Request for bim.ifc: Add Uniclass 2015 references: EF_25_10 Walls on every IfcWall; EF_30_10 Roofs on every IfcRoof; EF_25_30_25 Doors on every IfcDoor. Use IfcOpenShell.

First a look at what the model holds.

```python
import ifcopenshell

model = ifcopenshell.open("bim.ifc")
print(model.schema)
print("classifications:", [c.Name for c in model.by_type("IfcClassification")])
for ifc_class in ("IfcDoor", "IfcRoof", "IfcStair", "IfcWall", "IfcWindow"):
    print(ifc_class, len(model.by_type(ifc_class)))
```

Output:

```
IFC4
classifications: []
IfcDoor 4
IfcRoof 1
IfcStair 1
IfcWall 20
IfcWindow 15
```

```python
import ifcopenshell
import ifcopenshell.api.classification

model = ifcopenshell.open("bim.ifc")

system = ifcopenshell.api.classification.add_classification(model, classification="Uniclass 2015")

codes = {
    "IfcWall": ("EF_25_10", "Walls"),
    "IfcRoof": ("EF_30_10", "Roofs"),
    "IfcDoor": ("EF_25_30_25", "Doors"),
}
for ifc_class, (code, name) in codes.items():
    products = model.by_type(ifc_class)
    ifcopenshell.api.classification.add_reference(
        model, products=products, classification=system, identification=code, name=name
    )
    print(code, len(products))

model.write("bim_rev.ifc")
```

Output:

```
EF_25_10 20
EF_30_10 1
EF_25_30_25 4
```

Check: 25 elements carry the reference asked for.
